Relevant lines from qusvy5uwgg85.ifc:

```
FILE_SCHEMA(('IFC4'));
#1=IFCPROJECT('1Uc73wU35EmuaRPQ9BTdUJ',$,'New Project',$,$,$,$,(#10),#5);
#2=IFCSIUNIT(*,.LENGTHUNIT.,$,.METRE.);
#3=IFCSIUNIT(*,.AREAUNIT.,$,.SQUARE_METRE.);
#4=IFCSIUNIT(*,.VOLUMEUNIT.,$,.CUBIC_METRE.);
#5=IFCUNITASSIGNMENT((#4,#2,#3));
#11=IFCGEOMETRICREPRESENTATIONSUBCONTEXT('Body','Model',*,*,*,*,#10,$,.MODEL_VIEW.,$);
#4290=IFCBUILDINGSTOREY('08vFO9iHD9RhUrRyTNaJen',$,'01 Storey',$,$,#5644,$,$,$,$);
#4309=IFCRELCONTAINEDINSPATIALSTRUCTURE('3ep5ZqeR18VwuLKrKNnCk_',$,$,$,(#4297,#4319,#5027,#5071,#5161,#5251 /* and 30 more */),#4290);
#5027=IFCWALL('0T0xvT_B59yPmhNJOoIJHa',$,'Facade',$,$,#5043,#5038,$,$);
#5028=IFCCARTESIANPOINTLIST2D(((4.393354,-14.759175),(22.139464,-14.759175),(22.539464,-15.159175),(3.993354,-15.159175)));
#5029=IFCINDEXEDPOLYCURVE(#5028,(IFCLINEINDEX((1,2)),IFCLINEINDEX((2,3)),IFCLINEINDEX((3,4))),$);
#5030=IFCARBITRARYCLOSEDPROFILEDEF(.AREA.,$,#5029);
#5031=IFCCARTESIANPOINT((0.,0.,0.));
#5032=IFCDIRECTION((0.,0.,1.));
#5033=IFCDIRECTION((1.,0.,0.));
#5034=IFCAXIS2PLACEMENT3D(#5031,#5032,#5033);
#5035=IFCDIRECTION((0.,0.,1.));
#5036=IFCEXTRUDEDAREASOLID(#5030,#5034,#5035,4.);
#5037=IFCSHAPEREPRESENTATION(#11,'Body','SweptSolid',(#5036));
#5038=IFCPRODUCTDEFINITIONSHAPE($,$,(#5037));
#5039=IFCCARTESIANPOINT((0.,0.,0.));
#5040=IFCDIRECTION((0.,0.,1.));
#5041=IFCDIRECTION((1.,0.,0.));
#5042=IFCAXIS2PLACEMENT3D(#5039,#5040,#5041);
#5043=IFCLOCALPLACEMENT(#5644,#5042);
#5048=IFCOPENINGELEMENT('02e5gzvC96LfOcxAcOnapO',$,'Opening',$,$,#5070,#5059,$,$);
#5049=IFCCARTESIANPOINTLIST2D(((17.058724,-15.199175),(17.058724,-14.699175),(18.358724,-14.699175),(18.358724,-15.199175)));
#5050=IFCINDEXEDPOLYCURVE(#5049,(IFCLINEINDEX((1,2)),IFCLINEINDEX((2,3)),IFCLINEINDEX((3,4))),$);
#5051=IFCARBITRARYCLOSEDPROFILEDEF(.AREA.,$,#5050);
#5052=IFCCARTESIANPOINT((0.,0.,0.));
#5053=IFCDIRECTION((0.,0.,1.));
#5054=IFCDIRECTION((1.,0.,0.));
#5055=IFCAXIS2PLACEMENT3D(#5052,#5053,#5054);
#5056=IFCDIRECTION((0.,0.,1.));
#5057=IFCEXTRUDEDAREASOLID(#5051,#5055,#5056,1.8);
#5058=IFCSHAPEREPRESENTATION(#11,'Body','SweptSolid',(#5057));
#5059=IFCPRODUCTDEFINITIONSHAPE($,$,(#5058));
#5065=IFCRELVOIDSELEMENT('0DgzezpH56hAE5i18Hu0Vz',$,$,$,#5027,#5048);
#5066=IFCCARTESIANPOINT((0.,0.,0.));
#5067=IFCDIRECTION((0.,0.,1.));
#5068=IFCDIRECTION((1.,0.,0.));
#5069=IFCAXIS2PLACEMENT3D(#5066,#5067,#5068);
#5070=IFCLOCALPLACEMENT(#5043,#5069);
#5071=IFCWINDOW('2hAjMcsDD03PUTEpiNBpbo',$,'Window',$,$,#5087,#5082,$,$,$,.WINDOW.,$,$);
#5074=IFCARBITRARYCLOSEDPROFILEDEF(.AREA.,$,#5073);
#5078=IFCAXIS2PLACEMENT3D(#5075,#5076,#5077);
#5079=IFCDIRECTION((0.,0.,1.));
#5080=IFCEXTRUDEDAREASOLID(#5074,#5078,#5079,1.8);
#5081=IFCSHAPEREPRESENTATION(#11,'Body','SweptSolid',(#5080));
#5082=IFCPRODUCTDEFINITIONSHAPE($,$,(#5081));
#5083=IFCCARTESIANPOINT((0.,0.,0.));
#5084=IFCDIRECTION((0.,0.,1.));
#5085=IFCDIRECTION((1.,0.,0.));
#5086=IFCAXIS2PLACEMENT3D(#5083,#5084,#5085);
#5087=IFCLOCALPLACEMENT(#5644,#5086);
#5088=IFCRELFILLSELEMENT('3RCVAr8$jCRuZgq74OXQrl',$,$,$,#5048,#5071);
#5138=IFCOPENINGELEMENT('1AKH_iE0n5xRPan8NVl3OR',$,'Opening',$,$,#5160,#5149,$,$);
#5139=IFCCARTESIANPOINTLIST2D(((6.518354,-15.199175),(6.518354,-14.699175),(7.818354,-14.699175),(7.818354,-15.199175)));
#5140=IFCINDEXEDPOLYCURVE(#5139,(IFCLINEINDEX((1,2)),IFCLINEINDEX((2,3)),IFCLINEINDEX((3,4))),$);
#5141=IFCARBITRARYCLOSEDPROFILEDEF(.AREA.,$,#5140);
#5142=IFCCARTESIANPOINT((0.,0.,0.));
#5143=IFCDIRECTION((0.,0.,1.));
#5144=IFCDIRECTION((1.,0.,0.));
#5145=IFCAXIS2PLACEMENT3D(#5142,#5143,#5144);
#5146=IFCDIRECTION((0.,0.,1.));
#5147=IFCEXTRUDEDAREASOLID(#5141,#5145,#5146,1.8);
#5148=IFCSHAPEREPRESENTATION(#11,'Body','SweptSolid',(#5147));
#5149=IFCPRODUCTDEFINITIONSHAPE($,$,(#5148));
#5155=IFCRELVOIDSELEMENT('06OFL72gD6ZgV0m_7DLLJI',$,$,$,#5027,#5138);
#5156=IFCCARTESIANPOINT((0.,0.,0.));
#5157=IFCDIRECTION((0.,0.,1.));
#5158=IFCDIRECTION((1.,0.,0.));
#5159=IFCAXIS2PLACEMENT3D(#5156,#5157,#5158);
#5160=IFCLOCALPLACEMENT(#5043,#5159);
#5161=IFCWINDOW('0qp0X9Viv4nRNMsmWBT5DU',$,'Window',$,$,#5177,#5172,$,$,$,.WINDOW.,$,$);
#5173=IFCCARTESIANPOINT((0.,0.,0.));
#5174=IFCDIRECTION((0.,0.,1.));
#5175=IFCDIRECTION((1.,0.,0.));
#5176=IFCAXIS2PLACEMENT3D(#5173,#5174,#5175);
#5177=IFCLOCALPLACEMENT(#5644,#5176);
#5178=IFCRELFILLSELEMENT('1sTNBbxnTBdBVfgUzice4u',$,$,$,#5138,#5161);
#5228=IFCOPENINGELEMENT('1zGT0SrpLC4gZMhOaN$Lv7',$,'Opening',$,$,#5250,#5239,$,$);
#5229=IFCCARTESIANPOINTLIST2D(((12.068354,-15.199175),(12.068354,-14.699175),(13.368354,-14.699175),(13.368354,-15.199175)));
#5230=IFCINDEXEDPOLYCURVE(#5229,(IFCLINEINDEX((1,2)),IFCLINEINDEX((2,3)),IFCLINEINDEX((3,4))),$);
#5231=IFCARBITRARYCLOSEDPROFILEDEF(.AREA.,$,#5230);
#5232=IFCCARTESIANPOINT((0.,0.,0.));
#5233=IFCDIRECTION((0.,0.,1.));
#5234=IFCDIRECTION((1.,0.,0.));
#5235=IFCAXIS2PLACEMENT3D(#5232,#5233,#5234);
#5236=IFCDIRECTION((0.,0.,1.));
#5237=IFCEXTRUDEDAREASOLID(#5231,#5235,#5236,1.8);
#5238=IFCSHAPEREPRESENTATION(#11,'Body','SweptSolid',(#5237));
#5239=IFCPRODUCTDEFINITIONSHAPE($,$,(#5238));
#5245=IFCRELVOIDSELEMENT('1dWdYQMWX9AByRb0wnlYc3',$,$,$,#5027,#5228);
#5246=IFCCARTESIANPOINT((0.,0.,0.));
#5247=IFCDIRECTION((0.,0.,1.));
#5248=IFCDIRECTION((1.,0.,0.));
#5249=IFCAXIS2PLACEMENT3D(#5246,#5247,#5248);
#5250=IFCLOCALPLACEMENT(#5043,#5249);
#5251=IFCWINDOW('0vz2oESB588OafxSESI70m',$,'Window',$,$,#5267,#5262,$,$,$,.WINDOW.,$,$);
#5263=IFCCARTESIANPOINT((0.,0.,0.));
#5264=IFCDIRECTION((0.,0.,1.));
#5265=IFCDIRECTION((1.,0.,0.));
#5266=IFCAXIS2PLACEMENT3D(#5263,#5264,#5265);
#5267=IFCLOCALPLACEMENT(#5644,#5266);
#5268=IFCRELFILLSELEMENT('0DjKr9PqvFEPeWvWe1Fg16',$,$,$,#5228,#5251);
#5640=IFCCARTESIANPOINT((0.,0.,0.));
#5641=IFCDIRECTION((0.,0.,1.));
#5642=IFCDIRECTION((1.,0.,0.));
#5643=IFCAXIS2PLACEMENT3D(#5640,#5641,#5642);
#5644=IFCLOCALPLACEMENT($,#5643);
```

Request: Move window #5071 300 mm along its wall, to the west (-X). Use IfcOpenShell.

```python
import ifcopenshell
import ifcopenshell.api.geometry
import ifcopenshell.util.placement

model = ifcopenshell.open("qusvy5uwgg85.ifc")

window = model.by_guid("2hAjMcsDD03PUTEpiNBpbo")
opening = window.FillsVoids[0].RelatingOpeningElement
wall = opening.VoidsElements[0].RelatingBuildingElement

wall_matrix = ifcopenshell.util.placement.get_local_placement(wall.ObjectPlacement)
shift = wall_matrix[:3, 0] * -0.3
before = ifcopenshell.util.placement.get_local_placement(window.ObjectPlacement)[:3, 3].copy()

# The window is not placed relative to its opening, so move both.
for product in (opening, window):
    matrix = ifcopenshell.util.placement.get_local_placement(product.ObjectPlacement)
    matrix[:3, 3] += shift
    ifcopenshell.api.geometry.edit_object_placement(model, product=product, matrix=matrix, is_si=False)

after = ifcopenshell.util.placement.get_local_placement(window.ObjectPlacement)[:3, 3]
print("window moved by", (after - before).round(3) + 0.0)

model.write("qusvy5uwgg85_edited.ifc")
```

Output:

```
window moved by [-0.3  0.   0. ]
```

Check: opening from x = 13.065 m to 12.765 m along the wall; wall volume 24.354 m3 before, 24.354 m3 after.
